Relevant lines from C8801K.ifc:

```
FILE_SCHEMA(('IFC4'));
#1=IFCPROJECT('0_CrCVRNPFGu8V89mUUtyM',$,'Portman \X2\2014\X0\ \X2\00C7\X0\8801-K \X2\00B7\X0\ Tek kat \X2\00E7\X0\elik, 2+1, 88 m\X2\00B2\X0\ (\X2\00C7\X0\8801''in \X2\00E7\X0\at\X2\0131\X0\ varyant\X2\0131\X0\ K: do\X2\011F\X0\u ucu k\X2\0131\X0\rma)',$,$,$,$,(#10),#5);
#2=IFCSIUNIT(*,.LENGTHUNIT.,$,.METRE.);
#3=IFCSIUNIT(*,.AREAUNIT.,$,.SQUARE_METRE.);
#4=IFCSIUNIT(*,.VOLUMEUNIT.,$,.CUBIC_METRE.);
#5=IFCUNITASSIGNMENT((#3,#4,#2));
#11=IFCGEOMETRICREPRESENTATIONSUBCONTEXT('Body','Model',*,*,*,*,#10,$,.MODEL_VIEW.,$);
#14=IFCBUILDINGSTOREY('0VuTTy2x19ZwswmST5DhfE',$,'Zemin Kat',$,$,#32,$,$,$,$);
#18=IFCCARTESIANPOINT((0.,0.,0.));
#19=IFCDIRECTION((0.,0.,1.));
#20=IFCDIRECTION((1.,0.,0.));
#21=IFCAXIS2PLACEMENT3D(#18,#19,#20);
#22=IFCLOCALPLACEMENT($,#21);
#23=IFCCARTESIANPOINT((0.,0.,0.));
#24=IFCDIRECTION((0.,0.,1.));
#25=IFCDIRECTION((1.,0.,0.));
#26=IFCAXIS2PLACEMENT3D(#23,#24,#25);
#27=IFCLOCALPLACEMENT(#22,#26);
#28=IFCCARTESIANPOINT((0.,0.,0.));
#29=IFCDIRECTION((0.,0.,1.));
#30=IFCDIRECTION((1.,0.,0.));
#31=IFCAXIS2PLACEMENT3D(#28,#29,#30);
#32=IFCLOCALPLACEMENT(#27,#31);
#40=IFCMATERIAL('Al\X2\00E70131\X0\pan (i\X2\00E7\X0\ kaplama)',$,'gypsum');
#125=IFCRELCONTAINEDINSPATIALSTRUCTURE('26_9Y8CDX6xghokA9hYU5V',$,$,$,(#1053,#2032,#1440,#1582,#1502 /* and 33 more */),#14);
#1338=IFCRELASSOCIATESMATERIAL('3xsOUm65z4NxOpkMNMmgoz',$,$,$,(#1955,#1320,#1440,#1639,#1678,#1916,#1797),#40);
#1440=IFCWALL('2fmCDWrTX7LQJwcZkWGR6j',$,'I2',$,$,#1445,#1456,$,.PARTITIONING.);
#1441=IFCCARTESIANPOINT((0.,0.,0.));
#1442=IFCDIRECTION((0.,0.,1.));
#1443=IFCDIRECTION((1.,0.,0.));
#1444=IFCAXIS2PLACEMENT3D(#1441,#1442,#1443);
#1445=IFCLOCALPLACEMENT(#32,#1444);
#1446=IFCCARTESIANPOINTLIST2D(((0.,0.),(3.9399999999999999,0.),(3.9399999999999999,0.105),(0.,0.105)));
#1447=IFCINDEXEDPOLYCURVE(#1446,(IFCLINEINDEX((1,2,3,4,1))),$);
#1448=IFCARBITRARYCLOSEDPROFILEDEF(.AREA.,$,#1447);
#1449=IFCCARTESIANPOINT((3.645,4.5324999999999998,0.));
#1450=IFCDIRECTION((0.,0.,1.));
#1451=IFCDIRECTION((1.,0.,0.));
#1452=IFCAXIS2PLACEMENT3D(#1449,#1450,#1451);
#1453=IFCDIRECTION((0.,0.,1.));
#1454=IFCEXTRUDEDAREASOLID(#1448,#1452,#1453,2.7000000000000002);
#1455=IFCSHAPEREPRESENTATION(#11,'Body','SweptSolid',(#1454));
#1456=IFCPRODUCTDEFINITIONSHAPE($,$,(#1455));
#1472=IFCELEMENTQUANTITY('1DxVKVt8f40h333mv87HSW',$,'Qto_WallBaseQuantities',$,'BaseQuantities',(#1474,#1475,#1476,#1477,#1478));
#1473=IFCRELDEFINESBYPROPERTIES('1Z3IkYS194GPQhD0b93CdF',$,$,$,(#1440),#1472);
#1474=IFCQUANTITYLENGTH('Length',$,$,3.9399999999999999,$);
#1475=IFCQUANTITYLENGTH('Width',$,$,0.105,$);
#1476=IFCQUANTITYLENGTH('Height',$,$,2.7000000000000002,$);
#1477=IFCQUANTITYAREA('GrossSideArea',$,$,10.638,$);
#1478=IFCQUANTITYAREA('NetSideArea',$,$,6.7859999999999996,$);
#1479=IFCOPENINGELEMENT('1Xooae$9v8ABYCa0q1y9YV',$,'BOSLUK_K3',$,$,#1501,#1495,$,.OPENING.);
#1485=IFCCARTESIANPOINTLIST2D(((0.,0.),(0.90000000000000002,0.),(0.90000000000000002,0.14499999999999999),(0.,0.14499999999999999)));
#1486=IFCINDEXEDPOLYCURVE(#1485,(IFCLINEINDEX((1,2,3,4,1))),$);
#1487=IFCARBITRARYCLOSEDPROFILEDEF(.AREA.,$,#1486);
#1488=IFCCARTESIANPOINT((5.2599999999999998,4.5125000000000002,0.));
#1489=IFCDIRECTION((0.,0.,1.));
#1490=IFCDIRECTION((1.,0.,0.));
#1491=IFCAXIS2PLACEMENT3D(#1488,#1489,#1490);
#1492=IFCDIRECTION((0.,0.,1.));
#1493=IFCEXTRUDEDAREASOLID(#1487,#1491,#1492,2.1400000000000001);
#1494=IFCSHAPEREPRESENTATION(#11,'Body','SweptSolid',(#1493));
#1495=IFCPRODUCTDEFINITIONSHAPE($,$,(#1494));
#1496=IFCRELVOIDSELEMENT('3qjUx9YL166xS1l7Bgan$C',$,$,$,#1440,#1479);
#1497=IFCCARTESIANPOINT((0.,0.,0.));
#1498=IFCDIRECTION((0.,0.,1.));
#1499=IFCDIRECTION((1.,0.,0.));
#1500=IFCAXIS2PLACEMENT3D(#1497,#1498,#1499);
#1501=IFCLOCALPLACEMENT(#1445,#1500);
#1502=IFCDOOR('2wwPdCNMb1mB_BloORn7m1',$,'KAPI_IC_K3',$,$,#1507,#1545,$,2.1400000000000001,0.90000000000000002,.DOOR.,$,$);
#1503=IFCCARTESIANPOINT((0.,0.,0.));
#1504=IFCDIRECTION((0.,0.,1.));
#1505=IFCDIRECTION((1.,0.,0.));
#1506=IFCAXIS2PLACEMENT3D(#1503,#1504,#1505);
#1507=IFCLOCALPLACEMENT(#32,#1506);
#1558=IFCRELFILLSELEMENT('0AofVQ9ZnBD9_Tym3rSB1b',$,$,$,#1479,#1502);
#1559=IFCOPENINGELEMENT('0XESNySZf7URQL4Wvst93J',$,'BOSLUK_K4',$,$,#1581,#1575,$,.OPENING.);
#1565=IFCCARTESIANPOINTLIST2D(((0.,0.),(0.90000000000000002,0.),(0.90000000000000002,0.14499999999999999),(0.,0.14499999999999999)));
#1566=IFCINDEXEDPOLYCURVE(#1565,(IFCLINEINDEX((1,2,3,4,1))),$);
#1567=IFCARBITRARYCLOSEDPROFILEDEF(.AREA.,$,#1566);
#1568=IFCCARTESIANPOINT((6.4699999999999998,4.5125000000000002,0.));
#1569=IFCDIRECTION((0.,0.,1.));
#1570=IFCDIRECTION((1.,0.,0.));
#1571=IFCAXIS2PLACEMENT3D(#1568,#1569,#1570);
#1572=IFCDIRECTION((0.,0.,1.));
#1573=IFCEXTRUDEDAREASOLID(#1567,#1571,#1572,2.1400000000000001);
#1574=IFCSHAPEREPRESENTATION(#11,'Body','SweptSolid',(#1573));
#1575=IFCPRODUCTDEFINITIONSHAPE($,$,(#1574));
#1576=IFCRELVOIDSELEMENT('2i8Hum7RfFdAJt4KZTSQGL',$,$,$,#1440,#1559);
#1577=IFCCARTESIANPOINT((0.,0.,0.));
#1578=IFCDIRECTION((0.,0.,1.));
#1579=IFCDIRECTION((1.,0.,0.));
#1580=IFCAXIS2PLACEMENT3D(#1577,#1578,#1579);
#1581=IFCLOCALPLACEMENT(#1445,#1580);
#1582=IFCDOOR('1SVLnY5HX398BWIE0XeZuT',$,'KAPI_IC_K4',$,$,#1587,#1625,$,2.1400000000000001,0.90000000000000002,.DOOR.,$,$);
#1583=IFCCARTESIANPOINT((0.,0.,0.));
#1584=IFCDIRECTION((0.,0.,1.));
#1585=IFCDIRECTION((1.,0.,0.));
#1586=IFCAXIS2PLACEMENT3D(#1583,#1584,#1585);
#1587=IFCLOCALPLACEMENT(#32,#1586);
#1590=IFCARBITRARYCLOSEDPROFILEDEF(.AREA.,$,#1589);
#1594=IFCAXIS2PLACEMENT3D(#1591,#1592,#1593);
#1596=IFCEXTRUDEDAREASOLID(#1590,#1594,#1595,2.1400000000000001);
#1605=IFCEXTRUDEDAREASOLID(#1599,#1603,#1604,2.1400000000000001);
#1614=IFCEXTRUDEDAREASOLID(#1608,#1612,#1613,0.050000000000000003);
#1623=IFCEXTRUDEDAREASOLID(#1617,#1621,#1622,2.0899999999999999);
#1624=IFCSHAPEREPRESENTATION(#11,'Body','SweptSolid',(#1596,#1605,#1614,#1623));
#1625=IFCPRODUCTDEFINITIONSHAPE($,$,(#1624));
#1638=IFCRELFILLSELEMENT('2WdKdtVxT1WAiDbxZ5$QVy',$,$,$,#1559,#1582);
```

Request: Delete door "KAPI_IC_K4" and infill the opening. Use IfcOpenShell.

```python
import ifcopenshell
import ifcopenshell.api.feature
import ifcopenshell.api.pset
import ifcopenshell.api.root
import ifcopenshell.geom
import ifcopenshell.util.element
import ifcopenshell.util.shape
import ifcopenshell.util.unit

model = ifcopenshell.open("C8801K.ifc")
area_scale = ifcopenshell.util.unit.calculate_unit_scale(model, "AREAUNIT")
settings = ifcopenshell.geom.settings()


def volume(element):
    """Net volume in cubic metres, openings subtracted."""
    shape = ifcopenshell.geom.create_shape(settings, element)
    return ifcopenshell.util.shape.get_volume(shape.geometry)


door = model.by_id(1582)
opening = door.FillsVoids[0].RelatingOpeningElement
wall = opening.VoidsElements[0].RelatingBuildingElement
before = volume(wall)

ifcopenshell.api.root.remove_product(model, product=door)
ifcopenshell.api.feature.remove_feature(model, feature=opening)

after = volume(wall)
thickness = 0.105  # wall thickness in metres

# Update the wall's stored quantities.
qto = model.by_id(ifcopenshell.util.element.get_pset(wall, "Qto_WallBaseQuantities", should_inherit=False)["id"])
ifcopenshell.api.pset.edit_qto(model, qto=qto, properties={"NetSideArea": after / thickness / area_scale})

print(f"wall volume {before:.3f} -> {after:.3f} m3")

model.write("C8801K_edited.ifc")
```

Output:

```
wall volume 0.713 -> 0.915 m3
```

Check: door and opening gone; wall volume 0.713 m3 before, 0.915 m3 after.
